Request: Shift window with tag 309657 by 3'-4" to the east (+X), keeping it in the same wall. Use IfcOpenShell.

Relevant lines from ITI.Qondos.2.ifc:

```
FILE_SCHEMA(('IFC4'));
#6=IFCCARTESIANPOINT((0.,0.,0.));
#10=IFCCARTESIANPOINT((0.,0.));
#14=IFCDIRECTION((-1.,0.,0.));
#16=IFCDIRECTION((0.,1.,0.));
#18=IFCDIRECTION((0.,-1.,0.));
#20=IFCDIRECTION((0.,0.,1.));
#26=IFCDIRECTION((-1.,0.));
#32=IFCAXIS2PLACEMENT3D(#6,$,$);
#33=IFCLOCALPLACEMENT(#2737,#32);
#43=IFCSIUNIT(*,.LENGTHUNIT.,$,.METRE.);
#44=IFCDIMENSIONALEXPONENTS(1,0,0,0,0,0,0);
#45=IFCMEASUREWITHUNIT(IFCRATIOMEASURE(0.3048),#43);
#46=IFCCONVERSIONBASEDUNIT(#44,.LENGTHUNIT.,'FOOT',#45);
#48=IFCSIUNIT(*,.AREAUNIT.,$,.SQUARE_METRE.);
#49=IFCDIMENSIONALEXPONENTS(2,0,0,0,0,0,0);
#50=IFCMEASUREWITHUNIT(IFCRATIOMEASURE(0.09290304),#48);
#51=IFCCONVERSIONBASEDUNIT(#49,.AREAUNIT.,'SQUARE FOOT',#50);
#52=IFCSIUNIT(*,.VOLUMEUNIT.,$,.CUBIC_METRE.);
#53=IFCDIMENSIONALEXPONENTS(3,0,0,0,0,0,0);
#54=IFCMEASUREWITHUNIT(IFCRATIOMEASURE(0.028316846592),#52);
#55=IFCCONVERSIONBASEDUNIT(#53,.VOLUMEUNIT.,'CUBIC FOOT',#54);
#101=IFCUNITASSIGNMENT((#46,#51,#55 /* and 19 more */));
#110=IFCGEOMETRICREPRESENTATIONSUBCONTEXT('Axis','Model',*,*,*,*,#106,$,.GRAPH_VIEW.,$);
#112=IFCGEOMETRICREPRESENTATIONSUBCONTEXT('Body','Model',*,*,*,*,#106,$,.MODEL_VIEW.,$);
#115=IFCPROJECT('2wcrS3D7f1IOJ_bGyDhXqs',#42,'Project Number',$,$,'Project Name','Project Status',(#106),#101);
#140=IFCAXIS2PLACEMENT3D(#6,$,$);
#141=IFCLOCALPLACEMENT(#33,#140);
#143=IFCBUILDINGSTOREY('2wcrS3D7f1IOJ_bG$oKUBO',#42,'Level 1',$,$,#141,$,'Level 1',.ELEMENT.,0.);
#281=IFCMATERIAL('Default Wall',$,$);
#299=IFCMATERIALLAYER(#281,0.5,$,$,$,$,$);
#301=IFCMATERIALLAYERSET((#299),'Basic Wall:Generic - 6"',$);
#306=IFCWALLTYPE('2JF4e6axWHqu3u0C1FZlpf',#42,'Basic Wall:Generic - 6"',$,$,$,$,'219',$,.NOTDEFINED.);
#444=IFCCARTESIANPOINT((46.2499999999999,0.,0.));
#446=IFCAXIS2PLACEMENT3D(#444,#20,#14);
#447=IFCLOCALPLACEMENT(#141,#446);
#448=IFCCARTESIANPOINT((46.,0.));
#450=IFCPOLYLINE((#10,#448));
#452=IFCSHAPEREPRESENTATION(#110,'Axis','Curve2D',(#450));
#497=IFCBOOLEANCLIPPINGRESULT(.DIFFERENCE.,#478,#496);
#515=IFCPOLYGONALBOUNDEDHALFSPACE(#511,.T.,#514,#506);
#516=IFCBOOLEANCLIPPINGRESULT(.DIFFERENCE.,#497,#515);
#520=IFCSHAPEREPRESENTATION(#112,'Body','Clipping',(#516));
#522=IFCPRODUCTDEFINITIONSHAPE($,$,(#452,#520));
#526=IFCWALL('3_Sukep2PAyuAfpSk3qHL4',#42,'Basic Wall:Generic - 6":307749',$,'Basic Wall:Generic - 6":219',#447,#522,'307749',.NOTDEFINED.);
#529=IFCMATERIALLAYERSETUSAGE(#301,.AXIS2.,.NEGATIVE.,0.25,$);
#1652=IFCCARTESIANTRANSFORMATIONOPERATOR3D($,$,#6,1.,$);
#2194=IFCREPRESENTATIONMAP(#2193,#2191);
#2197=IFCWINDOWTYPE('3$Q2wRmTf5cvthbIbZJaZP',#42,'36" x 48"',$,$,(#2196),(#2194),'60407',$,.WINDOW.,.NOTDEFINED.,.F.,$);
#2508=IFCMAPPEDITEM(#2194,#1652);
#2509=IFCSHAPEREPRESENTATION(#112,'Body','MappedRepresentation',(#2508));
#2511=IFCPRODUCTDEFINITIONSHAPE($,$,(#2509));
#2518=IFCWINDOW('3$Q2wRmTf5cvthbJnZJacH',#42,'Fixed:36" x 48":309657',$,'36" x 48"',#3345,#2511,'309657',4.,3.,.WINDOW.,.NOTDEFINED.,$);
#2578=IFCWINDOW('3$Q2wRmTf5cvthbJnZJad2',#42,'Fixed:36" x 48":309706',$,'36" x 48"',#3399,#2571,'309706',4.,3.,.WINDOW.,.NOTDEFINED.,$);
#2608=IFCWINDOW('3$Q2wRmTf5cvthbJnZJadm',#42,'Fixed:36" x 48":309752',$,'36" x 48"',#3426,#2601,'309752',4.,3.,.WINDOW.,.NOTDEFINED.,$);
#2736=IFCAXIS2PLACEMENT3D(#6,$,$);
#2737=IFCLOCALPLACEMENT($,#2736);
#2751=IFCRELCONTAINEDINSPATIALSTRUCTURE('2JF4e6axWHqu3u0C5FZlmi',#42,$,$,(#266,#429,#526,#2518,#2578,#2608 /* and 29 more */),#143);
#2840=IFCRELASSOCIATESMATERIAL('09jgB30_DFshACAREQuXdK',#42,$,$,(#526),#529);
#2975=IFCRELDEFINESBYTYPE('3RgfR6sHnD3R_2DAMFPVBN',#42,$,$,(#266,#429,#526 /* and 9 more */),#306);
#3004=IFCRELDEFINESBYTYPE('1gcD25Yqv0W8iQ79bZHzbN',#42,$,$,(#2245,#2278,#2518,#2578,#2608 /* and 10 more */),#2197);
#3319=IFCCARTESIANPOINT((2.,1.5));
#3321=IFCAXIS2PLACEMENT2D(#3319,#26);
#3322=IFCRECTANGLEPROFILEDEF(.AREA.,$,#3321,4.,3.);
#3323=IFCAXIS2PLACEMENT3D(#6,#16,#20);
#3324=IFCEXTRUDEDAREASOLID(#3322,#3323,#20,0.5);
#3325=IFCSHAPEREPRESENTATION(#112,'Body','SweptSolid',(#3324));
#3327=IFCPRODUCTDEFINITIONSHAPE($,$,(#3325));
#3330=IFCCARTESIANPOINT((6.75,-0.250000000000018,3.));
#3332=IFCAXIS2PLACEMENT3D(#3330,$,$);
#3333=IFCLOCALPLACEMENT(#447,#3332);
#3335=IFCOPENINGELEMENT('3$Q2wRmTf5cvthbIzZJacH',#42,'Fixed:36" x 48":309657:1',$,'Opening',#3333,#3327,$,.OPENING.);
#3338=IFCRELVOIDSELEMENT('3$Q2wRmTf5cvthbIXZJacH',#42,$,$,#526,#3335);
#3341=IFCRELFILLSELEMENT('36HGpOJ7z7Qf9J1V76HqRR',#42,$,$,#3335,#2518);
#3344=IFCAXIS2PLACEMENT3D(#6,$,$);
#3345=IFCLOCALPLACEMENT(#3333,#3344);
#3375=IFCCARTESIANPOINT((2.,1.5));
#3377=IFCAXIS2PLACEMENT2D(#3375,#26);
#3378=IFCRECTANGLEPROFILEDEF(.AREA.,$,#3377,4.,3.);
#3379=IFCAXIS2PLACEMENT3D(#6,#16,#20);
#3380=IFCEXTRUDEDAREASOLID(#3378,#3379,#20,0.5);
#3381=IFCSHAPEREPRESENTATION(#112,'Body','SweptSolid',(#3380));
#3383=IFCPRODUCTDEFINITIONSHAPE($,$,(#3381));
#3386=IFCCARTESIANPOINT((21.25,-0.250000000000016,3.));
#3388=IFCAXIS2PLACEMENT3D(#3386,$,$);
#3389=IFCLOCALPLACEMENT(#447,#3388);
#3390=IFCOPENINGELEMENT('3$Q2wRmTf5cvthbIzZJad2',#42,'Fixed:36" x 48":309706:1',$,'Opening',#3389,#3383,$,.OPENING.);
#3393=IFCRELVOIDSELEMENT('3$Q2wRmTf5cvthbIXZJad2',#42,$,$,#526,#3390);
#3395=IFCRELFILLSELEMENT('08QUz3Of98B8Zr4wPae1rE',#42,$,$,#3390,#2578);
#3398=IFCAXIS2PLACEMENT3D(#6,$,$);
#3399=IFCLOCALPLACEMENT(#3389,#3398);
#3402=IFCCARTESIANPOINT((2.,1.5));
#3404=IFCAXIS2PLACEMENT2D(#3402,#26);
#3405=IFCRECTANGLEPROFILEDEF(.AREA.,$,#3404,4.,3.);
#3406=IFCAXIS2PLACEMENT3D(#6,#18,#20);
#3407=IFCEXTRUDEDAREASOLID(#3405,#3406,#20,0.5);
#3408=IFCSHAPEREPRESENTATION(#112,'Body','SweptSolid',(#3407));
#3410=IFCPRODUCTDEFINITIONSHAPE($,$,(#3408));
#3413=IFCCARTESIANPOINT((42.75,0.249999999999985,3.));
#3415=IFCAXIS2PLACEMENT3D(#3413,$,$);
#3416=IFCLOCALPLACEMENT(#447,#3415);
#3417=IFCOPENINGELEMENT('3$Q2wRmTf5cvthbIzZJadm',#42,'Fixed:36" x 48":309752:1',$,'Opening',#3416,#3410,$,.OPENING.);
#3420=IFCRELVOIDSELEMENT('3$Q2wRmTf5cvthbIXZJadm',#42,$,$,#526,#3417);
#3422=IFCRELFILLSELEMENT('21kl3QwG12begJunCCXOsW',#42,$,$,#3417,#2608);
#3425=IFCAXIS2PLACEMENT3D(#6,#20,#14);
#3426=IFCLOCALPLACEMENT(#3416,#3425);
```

```python
import ifcopenshell
import ifcopenshell.api.geometry
import ifcopenshell.util.placement
import ifcopenshell.util.unit

model = ifcopenshell.open("ITI.Qondos.2.ifc")
unit_scale = ifcopenshell.util.unit.calculate_unit_scale(model)

window = model.by_guid("3$Q2wRmTf5cvthbJnZJacH")
opening = window.FillsVoids[0].RelatingOpeningElement
wall = opening.VoidsElements[0].RelatingBuildingElement

wall_matrix = ifcopenshell.util.placement.get_local_placement(wall.ObjectPlacement)
shift = wall_matrix[:3, 0] * -40 * 0.0254 / unit_scale
before = ifcopenshell.util.placement.get_local_placement(window.ObjectPlacement)[:3, 3].copy()

# The window is placed relative to its opening, so it follows when the opening moves.
matrix = ifcopenshell.util.placement.get_local_placement(opening.ObjectPlacement)
matrix[:3, 3] += shift
ifcopenshell.api.geometry.edit_object_placement(
    model, product=opening, matrix=matrix, is_si=False, should_transform_children=True
)

after = ifcopenshell.util.placement.get_local_placement(window.ObjectPlacement)[:3, 3]
print("window moved by", (after - before).round(3) + 0.0)

model.write("ITI.Qondos.2_edited.ifc")
```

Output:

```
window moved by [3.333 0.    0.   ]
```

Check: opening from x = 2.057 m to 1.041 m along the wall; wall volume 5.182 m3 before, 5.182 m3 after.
